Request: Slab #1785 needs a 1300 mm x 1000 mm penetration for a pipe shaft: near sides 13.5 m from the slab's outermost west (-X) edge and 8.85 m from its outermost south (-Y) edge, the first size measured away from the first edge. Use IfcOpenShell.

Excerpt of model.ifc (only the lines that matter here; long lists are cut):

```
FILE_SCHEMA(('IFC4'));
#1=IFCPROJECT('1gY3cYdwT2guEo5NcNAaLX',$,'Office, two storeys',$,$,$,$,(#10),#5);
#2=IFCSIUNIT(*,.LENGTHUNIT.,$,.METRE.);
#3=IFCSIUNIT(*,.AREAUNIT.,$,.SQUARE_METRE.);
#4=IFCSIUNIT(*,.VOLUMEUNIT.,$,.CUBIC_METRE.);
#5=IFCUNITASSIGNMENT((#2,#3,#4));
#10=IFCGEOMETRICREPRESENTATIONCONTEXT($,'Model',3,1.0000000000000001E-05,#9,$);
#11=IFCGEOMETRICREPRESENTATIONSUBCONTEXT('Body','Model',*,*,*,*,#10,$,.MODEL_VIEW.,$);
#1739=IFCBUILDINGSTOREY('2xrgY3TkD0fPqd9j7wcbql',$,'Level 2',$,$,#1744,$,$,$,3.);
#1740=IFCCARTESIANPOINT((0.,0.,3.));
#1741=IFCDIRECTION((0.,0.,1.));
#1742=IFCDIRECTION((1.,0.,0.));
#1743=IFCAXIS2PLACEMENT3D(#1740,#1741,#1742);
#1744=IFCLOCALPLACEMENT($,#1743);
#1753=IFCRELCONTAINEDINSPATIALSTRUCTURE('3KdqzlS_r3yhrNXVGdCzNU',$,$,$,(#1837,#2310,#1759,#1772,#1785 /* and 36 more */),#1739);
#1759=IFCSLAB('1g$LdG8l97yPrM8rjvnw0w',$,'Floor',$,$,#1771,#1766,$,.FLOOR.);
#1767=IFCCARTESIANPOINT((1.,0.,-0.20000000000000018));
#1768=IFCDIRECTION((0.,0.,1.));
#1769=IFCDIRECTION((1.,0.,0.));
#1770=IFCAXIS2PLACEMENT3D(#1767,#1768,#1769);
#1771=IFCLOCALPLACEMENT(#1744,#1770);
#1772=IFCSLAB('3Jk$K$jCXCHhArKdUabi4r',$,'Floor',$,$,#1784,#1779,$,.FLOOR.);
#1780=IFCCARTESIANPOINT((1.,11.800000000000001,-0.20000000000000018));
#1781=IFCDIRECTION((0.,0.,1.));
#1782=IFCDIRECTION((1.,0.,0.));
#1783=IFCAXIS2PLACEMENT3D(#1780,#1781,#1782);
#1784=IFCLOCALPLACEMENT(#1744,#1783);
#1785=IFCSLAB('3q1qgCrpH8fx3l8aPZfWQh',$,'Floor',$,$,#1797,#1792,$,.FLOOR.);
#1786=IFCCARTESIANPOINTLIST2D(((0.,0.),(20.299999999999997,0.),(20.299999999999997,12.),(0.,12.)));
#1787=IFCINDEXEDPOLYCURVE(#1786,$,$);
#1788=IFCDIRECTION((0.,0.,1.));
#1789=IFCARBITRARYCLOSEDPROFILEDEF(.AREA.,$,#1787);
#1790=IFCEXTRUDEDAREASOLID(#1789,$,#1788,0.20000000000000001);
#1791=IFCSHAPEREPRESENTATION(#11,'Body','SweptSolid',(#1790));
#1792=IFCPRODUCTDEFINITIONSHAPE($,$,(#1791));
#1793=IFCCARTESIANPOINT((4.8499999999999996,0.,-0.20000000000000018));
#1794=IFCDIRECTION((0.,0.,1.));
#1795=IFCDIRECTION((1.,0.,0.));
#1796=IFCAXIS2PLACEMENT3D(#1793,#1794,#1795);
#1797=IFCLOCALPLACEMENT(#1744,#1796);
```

```python
import numpy as np
import ifcopenshell
import ifcopenshell.api.feature
import ifcopenshell.api.geometry
import ifcopenshell.api.root
import ifcopenshell.geom
import ifcopenshell.util.placement
import ifcopenshell.util.representation
import ifcopenshell.util.shape
import ifcopenshell.util.unit

model = ifcopenshell.open("model.ifc")
unit_scale = ifcopenshell.util.unit.calculate_unit_scale(model)
settings = ifcopenshell.geom.settings()


def volume(element):
    """Net volume in cubic metres, openings subtracted."""
    shape = ifcopenshell.geom.create_shape(settings, element)
    return ifcopenshell.util.shape.get_volume(shape.geometry)


slab = model.by_guid("3q1qgCrpH8fx3l8aPZfWQh")
before = volume(slab)

# Extent in the slab's own axes, in metres. The edges named are its -X and -Y sides.
slab_shape = ifcopenshell.geom.create_shape(settings, slab)
vertices = ifcopenshell.util.shape.get_vertices(slab_shape.geometry)
x_min, y_min, bottom = vertices.min(axis=0)
top = vertices[:, 2].max()

opening = ifcopenshell.api.root.create_entity(model, ifc_class="IfcOpeningElement", name="Pipe shaft opening", predefined_type="OPENING")
context = ifcopenshell.util.representation.get_context(model, "Model", "Body", "MODEL_VIEW")
width, depth = 1.3, 1
outline = [(0.0, 0.0), (width, 0.0), (width, depth), (0.0, depth), (0.0, 0.0)]
# Overshoot both faces by 50 mm so the cut is clean.
shape = ifcopenshell.api.geometry.add_slab_representation(
    model, context=context, depth=top - bottom + 0.1, polyline=outline
)
ifcopenshell.api.geometry.assign_representation(model, product=opening, representation=shape)

matrix = ifcopenshell.util.placement.get_local_placement(slab.ObjectPlacement)
matrix[:, 3] = matrix @ np.append(np.array([x_min + 13.5, y_min + 8.85, bottom - 0.05]) / unit_scale, 1.0)
ifcopenshell.api.geometry.edit_object_placement(model, product=opening, matrix=matrix, is_si=False)
ifcopenshell.api.feature.add_feature(model, feature=opening, element=slab)

after = volume(slab)

print(f"slab volume {before:.3f} -> {after:.3f} m3")

model.write("model_updated.ifc")
```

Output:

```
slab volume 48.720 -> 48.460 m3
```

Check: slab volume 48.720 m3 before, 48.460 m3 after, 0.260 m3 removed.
